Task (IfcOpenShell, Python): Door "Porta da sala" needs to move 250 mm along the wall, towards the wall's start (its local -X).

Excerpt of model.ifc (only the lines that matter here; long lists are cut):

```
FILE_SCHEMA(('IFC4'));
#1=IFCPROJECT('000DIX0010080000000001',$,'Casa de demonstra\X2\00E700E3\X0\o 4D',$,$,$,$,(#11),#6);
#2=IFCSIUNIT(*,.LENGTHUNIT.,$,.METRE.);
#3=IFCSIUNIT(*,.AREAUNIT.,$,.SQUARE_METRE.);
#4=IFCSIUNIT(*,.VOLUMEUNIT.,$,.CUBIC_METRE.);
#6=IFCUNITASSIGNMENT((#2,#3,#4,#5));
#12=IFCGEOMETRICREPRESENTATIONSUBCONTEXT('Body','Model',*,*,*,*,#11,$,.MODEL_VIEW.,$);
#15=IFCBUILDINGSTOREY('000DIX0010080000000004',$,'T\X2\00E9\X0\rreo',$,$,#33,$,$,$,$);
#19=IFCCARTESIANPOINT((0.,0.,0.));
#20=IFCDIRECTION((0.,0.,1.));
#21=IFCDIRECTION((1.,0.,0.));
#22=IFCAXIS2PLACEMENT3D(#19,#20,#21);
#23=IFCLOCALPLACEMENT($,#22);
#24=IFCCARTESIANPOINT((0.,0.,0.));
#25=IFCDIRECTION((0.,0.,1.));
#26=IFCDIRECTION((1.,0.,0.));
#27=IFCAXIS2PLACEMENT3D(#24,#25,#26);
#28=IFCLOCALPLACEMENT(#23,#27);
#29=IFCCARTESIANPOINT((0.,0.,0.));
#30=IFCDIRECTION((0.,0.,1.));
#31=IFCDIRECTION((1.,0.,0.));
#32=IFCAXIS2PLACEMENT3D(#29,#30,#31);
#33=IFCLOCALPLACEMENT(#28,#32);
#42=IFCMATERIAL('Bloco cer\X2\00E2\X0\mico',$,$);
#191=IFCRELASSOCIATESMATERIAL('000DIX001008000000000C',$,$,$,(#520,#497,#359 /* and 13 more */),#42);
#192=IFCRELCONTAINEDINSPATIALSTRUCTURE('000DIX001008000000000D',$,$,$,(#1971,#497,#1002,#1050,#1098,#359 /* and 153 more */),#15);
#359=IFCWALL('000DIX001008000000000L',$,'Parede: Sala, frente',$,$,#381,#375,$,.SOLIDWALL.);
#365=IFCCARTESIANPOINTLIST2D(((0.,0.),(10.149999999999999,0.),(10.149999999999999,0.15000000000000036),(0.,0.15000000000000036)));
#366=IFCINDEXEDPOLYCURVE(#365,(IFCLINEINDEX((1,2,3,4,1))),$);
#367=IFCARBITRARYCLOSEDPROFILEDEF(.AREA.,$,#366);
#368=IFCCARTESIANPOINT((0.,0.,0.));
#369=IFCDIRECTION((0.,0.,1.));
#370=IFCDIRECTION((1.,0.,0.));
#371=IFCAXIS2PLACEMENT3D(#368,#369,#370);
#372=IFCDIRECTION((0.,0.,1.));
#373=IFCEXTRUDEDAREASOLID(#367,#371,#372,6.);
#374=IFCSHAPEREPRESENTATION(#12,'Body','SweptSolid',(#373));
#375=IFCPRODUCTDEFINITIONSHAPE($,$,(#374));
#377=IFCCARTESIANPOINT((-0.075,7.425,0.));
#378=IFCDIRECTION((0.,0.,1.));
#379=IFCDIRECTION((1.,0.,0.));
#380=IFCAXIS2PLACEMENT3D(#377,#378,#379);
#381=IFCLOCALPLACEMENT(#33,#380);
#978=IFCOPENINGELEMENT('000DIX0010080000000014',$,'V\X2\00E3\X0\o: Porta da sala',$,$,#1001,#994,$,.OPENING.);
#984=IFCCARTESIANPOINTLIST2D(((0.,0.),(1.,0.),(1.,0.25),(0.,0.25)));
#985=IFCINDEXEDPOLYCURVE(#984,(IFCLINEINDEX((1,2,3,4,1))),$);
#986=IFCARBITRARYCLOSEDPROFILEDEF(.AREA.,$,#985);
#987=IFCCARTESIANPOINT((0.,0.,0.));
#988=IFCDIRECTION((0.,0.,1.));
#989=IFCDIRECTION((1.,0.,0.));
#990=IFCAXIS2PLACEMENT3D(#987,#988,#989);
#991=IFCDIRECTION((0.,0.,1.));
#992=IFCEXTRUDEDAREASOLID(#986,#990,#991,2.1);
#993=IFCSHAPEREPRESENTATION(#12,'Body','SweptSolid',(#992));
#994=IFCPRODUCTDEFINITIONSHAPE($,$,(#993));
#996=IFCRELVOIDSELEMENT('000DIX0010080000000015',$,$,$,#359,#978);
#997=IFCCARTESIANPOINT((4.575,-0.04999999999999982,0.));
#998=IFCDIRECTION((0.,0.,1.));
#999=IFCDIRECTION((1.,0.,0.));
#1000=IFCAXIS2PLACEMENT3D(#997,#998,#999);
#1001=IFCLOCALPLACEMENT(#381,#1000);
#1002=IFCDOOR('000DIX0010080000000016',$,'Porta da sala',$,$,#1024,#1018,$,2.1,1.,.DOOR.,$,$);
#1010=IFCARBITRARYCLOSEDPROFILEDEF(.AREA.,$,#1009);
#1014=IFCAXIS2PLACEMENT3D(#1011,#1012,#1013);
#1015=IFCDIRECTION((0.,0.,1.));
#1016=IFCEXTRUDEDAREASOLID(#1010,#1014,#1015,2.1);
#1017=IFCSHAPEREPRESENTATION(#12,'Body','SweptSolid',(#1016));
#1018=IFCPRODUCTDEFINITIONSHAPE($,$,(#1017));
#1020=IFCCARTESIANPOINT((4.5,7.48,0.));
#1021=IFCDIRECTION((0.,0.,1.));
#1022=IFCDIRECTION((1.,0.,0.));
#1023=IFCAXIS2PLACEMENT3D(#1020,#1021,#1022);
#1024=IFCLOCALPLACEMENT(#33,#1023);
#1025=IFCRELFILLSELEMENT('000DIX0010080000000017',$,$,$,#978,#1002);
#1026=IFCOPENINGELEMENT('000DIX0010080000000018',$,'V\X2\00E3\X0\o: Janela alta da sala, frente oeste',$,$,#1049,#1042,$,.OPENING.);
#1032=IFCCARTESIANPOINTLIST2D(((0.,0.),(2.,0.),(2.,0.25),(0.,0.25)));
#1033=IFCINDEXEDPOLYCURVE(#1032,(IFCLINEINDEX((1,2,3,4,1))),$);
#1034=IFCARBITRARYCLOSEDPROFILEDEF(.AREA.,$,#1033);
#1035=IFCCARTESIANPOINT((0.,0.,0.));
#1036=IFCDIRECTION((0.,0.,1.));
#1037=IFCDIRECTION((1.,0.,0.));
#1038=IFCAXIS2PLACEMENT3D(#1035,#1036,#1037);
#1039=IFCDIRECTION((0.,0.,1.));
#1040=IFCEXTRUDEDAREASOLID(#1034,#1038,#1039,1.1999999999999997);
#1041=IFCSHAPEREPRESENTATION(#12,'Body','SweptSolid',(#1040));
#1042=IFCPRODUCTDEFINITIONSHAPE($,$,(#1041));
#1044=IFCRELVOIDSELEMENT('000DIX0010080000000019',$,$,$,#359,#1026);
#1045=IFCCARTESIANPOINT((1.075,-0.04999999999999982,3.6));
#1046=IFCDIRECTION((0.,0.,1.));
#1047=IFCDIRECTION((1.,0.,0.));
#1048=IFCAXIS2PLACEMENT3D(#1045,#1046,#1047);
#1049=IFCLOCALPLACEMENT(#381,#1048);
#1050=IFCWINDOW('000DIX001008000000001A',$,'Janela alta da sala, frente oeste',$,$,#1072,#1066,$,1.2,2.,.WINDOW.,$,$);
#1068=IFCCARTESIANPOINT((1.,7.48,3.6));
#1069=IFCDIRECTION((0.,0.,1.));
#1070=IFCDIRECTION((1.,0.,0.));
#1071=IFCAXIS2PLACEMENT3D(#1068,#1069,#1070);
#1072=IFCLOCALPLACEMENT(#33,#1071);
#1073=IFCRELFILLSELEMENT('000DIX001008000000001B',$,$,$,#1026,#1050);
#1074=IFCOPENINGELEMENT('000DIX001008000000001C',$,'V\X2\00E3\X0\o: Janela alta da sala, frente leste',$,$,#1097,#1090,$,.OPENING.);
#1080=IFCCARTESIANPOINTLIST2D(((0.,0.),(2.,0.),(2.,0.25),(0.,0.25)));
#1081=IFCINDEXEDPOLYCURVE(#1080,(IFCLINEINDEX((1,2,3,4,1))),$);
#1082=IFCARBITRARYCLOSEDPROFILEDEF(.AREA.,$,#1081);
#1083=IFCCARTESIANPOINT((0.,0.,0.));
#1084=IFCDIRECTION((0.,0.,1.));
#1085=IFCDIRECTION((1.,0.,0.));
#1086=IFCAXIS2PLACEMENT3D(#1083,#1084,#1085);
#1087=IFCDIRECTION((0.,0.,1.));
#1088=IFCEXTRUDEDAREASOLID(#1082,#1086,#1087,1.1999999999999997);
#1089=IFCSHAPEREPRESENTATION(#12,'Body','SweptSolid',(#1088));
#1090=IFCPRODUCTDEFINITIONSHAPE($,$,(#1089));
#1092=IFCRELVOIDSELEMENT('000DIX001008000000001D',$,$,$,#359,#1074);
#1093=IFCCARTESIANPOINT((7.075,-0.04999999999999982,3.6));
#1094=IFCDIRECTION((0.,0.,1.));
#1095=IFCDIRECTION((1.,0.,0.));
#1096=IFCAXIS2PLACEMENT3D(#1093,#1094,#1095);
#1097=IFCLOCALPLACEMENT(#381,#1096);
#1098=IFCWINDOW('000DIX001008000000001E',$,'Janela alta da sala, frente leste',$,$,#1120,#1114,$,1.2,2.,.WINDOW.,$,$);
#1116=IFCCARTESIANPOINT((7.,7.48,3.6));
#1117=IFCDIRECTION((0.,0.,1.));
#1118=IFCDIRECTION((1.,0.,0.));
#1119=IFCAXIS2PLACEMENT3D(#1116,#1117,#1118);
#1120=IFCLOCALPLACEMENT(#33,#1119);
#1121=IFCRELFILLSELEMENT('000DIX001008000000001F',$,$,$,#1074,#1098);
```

```python
import ifcopenshell
import ifcopenshell.api.geometry
import ifcopenshell.util.placement
import ifcopenshell.util.unit

model = ifcopenshell.open("model.ifc")
unit_scale = ifcopenshell.util.unit.calculate_unit_scale(model)

door = model.by_guid("000DIX0010080000000016")
opening = door.FillsVoids[0].RelatingOpeningElement
wall = opening.VoidsElements[0].RelatingBuildingElement

wall_matrix = ifcopenshell.util.placement.get_local_placement(wall.ObjectPlacement)
shift = wall_matrix[:3, 0] * -0.25 / unit_scale
before = ifcopenshell.util.placement.get_local_placement(door.ObjectPlacement)[:3, 3].copy()

# The door is not placed relative to its opening, so move both.
for product in (opening, door):
    matrix = ifcopenshell.util.placement.get_local_placement(product.ObjectPlacement)
    matrix[:3, 3] += shift
    ifcopenshell.api.geometry.edit_object_placement(model, product=product, matrix=matrix, is_si=False)

after = ifcopenshell.util.placement.get_local_placement(door.ObjectPlacement)[:3, 3]
print("door moved by", (after - before).round(3) + 0.0)

model.write("model_edited.ifc")
```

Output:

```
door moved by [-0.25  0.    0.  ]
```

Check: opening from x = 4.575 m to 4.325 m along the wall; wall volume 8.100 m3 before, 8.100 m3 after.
